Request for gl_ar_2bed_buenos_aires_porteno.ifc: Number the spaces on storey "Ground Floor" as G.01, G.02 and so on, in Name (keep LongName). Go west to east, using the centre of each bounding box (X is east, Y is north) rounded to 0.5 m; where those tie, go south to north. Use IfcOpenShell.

First a look at what the model holds.

```python
import ifcopenshell
import ifcopenshell.util.element
import ifcopenshell.util.placement

model = ifcopenshell.open("gl_ar_2bed_buenos_aires_porteno.ifc")
print(model.schema)
storey = next(s for s in model.by_type("IfcBuildingStorey") if s.Name == "Ground Floor")
spaces = [e for e in ifcopenshell.util.element.get_decomposition(storey) if e.is_a("IfcSpace")]
for e in sorted(spaces, key=lambda e: e.id()):
    origin = ifcopenshell.util.placement.get_local_placement(e.ObjectPlacement)[:3, 3]
    print(e.id(), e.Name, e.LongName, origin.round(2) + 0.0, sep=" | ")
```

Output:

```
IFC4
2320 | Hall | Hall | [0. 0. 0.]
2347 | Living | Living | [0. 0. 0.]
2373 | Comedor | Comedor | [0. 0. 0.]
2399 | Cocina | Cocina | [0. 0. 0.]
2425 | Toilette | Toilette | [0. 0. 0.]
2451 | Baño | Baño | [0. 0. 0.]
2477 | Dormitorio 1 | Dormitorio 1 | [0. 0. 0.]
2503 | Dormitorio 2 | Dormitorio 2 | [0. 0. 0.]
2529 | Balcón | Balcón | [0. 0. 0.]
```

```python
import ifcopenshell
import ifcopenshell.geom
import ifcopenshell.util.element
import ifcopenshell.util.shape

model = ifcopenshell.open("gl_ar_2bed_buenos_aires_porteno.ifc")
settings = ifcopenshell.geom.settings()
settings.set("use-world-coords", True)


def centre(element):
    shape = ifcopenshell.geom.create_shape(settings, element)
    return ifcopenshell.util.shape.get_bbox_centroid(shape.geometry)


storey = next(s for s in model.by_type("IfcBuildingStorey") if s.Name == "Ground Floor")
spaces = [e for e in ifcopenshell.util.element.get_decomposition(storey) if e.is_a("IfcSpace")]

# Insertion points can sit at a corner or the storey origin, so sort by the geometry (in metres).
centres = {e: centre(e) for e in spaces}
spaces.sort(key=lambda e: (round(centres[e][0] / 0.5), centres[e][1]))

for i, e in enumerate(spaces, start=1):
    number = f"G.{i:02d}"
    e.Name = number
    print(e.id(), number)

model.write("gl_ar_2bed_buenos_aires_porteno_updated.ifc")
```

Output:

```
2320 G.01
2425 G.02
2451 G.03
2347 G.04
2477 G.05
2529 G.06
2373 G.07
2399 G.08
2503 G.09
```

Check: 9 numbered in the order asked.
